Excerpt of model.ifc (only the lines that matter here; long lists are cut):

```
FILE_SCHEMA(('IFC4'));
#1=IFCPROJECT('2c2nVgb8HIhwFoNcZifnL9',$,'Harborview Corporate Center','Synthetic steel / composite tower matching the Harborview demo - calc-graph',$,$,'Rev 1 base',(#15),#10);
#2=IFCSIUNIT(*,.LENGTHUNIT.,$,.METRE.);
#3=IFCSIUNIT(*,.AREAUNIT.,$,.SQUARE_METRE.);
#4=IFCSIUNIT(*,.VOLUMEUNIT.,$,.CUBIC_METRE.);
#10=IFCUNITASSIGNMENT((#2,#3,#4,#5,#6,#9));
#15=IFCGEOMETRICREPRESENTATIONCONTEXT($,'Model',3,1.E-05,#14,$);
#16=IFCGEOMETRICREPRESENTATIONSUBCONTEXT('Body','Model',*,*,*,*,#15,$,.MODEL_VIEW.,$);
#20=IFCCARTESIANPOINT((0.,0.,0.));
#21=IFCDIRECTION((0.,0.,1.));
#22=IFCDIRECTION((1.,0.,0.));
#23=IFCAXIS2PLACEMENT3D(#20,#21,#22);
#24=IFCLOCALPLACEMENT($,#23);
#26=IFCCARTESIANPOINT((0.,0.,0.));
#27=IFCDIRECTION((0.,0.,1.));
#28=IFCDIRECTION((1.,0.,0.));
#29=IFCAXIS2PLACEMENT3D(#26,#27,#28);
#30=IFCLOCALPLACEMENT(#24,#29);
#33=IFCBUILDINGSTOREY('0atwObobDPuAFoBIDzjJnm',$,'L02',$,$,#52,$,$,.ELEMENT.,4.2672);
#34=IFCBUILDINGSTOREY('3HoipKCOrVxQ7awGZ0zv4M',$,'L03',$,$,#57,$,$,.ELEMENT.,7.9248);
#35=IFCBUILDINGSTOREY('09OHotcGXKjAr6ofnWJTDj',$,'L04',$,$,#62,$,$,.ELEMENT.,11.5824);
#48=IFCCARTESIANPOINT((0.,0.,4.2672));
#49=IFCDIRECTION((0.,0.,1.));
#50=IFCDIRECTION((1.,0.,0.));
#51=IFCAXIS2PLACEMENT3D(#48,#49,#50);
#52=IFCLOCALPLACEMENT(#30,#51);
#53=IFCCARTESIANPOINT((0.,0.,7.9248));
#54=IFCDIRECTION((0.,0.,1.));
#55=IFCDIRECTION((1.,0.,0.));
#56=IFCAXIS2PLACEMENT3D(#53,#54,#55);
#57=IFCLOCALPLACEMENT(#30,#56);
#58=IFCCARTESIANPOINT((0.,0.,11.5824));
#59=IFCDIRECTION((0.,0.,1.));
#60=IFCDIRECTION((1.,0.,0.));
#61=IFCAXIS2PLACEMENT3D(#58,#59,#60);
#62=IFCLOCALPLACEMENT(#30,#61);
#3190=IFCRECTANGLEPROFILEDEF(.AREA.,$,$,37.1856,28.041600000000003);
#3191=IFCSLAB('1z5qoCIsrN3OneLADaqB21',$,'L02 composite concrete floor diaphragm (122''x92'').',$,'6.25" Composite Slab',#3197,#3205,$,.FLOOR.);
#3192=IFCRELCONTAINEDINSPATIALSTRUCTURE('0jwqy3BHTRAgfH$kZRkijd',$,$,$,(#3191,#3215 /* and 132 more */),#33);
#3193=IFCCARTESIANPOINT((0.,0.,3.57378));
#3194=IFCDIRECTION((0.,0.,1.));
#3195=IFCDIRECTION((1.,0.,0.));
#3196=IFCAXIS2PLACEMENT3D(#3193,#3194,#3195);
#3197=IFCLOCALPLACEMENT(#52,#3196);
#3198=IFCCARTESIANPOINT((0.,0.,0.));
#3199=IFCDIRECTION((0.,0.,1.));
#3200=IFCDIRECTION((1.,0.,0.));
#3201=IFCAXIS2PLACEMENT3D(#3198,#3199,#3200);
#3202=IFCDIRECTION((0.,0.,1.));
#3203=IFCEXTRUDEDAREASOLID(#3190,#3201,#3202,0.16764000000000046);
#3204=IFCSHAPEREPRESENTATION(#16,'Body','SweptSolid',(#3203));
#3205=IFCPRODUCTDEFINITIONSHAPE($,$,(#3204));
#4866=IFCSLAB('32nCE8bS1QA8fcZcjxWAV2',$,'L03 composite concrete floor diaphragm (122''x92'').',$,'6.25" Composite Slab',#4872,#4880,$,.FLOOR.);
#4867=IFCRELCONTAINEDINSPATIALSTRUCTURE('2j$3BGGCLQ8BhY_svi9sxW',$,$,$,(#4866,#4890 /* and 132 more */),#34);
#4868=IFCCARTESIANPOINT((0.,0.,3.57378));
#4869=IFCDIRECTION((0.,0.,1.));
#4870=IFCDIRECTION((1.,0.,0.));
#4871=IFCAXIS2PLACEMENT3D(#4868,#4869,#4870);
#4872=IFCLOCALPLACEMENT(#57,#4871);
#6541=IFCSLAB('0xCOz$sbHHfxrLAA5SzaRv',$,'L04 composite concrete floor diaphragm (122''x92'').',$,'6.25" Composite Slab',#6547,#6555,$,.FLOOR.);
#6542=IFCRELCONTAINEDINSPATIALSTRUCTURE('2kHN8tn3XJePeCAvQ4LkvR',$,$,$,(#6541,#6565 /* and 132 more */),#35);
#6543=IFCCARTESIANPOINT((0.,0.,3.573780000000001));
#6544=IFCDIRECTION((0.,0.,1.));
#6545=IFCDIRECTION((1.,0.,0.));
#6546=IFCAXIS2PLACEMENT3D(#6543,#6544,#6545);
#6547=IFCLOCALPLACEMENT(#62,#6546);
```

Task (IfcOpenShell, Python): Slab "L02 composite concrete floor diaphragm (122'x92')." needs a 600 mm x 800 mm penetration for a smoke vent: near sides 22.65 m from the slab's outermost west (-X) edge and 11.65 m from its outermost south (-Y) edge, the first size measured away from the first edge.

```python
import numpy as np
import ifcopenshell
import ifcopenshell.api.feature
import ifcopenshell.api.geometry
import ifcopenshell.api.root
import ifcopenshell.geom
import ifcopenshell.util.placement
import ifcopenshell.util.representation
import ifcopenshell.util.shape
import ifcopenshell.util.unit

model = ifcopenshell.open("model.ifc")
unit_scale = ifcopenshell.util.unit.calculate_unit_scale(model)
settings = ifcopenshell.geom.settings()


def volume(element):
    """Net volume in cubic metres, openings subtracted."""
    shape = ifcopenshell.geom.create_shape(settings, element)
    return ifcopenshell.util.shape.get_volume(shape.geometry)


slab = model.by_guid("1z5qoCIsrN3OneLADaqB21")
before = volume(slab)

# Extent in the slab's own axes, in metres. The edges named are its -X and -Y sides.
slab_shape = ifcopenshell.geom.create_shape(settings, slab)
vertices = ifcopenshell.util.shape.get_vertices(slab_shape.geometry)
x_min, y_min, bottom = vertices.min(axis=0)
top = vertices[:, 2].max()

opening = ifcopenshell.api.root.create_entity(model, ifc_class="IfcOpeningElement", name="Smoke vent opening", predefined_type="OPENING")
context = ifcopenshell.util.representation.get_context(model, "Model", "Body", "MODEL_VIEW")
width, depth = 0.6, 0.8
outline = [(0.0, 0.0), (width, 0.0), (width, depth), (0.0, depth), (0.0, 0.0)]
# Overshoot both faces by 50 mm so the cut is clean.
shape = ifcopenshell.api.geometry.add_slab_representation(
    model, context=context, depth=top - bottom + 0.1, polyline=outline
)
ifcopenshell.api.geometry.assign_representation(model, product=opening, representation=shape)

matrix = ifcopenshell.util.placement.get_local_placement(slab.ObjectPlacement)
matrix[:, 3] = matrix @ np.append(np.array([x_min + 22.65, y_min + 11.65, bottom - 0.05]) / unit_scale, 1.0)
ifcopenshell.api.geometry.edit_object_placement(model, product=opening, matrix=matrix, is_si=False)
ifcopenshell.api.feature.add_feature(model, feature=opening, element=slab)

after = volume(slab)

print(f"slab volume {before:.3f} -> {after:.3f} m3")

model.write("model_edited.ifc")
```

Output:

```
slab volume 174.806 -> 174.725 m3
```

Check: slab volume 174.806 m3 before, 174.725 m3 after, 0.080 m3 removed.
